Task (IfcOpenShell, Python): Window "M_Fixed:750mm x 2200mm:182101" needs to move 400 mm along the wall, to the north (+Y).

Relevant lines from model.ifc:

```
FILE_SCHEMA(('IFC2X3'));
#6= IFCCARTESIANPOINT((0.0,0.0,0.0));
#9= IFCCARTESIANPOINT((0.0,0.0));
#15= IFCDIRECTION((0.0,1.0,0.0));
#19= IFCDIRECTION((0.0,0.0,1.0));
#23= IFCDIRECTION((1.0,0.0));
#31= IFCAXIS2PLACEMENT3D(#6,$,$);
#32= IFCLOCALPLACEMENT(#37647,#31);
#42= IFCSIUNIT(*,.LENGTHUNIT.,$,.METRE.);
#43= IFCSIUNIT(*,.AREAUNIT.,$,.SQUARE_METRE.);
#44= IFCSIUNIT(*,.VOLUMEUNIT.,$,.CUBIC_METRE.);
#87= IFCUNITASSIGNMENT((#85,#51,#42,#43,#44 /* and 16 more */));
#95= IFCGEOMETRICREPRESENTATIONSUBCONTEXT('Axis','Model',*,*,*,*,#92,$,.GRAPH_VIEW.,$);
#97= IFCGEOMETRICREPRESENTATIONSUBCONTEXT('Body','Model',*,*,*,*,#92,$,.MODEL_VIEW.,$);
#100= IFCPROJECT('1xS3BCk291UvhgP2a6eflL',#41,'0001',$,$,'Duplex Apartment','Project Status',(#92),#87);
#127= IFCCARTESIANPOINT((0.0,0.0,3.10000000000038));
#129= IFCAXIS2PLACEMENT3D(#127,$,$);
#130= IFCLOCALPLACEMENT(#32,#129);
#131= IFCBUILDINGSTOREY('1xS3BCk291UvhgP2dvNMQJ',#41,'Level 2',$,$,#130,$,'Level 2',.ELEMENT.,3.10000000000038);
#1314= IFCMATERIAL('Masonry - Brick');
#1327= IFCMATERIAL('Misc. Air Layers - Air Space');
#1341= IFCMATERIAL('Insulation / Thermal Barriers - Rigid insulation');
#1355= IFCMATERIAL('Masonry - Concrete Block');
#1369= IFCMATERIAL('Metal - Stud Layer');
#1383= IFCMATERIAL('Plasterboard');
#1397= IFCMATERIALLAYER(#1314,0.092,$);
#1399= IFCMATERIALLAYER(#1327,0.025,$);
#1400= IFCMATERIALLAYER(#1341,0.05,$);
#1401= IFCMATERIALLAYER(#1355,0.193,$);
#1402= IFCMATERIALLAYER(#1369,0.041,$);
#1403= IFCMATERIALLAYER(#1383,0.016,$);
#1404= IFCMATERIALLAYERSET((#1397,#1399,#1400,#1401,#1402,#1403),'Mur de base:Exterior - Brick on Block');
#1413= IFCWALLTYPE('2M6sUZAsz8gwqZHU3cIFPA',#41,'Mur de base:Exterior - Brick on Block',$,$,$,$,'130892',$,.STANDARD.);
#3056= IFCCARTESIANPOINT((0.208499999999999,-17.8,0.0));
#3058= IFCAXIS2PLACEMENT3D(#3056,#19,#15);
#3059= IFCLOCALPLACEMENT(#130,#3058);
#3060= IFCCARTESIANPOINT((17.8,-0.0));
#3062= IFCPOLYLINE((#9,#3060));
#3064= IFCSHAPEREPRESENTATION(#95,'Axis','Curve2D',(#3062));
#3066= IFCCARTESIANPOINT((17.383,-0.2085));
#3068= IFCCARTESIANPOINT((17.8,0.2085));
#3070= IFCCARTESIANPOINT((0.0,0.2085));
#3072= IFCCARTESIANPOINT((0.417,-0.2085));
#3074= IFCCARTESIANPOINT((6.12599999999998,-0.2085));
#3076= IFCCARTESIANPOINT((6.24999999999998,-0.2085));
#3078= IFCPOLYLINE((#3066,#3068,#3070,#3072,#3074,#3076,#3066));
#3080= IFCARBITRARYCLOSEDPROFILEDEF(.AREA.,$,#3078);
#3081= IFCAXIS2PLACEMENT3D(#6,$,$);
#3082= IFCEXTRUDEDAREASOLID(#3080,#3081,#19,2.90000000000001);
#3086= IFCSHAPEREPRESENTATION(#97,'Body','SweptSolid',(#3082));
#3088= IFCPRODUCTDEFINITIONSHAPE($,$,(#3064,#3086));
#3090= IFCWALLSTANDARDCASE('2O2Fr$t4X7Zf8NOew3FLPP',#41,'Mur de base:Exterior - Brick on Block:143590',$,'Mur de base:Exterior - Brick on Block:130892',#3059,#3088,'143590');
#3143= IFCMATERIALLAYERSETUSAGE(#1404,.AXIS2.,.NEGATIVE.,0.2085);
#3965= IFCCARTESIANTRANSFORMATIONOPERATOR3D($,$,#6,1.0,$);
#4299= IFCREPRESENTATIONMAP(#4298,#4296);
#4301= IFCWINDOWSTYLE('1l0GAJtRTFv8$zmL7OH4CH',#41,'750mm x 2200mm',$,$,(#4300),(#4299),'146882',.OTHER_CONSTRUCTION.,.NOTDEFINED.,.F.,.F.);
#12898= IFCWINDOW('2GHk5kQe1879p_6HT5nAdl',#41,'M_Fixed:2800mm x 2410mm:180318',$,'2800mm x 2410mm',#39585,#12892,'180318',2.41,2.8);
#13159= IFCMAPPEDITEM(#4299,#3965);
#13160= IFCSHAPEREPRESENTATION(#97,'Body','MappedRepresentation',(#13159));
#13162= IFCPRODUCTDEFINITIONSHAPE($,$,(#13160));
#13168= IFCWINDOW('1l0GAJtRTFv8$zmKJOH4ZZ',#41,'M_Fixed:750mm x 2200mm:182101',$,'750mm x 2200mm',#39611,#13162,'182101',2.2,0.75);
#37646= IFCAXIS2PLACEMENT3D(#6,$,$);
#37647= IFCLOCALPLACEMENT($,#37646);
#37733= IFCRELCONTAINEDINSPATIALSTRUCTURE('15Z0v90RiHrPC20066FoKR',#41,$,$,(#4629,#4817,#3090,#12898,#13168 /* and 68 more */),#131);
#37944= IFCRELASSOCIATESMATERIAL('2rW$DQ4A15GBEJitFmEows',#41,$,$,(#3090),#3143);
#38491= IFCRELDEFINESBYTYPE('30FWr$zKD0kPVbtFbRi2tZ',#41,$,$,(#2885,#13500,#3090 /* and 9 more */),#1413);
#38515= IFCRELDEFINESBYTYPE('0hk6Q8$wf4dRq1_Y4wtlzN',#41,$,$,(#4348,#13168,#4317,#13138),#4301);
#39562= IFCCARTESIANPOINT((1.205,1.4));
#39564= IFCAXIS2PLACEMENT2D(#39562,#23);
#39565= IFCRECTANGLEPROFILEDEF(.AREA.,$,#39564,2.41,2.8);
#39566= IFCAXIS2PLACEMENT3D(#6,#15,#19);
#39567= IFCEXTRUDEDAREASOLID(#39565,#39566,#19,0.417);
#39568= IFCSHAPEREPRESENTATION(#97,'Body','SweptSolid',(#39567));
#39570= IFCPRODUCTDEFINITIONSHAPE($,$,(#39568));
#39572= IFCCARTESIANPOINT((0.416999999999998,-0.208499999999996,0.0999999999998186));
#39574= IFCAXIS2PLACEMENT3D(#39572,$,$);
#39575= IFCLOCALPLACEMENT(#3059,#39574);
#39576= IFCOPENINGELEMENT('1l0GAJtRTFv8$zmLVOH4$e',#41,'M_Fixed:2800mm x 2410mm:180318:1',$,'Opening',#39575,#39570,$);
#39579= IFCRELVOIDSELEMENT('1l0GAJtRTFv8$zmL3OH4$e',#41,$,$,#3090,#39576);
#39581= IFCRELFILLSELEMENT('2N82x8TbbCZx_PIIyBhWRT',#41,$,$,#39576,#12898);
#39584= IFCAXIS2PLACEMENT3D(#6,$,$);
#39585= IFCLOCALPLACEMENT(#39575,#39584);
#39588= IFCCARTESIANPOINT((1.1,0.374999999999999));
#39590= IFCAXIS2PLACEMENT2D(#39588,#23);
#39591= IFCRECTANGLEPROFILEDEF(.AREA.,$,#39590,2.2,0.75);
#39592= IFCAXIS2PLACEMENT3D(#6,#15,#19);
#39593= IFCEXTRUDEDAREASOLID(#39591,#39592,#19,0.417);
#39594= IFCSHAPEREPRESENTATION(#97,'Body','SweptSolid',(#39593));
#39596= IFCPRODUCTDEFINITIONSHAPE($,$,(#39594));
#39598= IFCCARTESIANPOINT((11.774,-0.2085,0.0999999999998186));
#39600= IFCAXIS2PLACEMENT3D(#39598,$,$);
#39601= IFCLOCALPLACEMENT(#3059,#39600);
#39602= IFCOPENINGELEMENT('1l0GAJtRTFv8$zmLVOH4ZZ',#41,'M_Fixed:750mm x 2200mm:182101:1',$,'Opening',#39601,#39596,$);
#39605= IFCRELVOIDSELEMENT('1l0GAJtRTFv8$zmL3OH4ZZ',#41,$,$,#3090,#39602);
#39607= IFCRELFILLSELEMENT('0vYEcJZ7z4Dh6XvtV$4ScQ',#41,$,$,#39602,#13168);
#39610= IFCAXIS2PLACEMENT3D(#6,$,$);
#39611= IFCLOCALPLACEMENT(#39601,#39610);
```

```python
import ifcopenshell
import ifcopenshell.api.geometry
import ifcopenshell.util.placement
import ifcopenshell.util.unit

model = ifcopenshell.open("model.ifc")
unit_scale = ifcopenshell.util.unit.calculate_unit_scale(model)

window = model.by_guid("1l0GAJtRTFv8$zmKJOH4ZZ")
opening = window.FillsVoids[0].RelatingOpeningElement
wall = opening.VoidsElements[0].RelatingBuildingElement

wall_matrix = ifcopenshell.util.placement.get_local_placement(wall.ObjectPlacement)
shift = wall_matrix[:3, 0] * 0.4 / unit_scale
before = ifcopenshell.util.placement.get_local_placement(window.ObjectPlacement)[:3, 3].copy()

# The window is placed relative to its opening, so it follows when the opening moves.
matrix = ifcopenshell.util.placement.get_local_placement(opening.ObjectPlacement)
matrix[:3, 3] += shift
ifcopenshell.api.geometry.edit_object_placement(
    model, product=opening, matrix=matrix, is_si=False, should_transform_children=True
)

after = ifcopenshell.util.placement.get_local_placement(window.ObjectPlacement)[:3, 3]
print("window moved by", (after - before).round(3) + 0.0)

model.write("model_edited.ifc")
```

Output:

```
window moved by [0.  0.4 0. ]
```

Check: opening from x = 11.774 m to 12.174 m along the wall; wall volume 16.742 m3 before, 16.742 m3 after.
